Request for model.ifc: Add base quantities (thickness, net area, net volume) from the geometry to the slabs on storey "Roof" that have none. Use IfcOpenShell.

First a look at what the model holds.

```python
import ifcopenshell
import ifcopenshell.util.element
import ifcopenshell.util.unit

model = ifcopenshell.open("model.ifc")
print(model.schema)
for unit_type in ("LENGTHUNIT", "AREAUNIT", "VOLUMEUNIT"):
    print(unit_type, ifcopenshell.util.unit.calculate_unit_scale(model, unit_type))
storey = next(s for s in model.by_type("IfcBuildingStorey") if s.Name == "Roof")
slabs = [e for e in ifcopenshell.util.element.get_decomposition(storey) if e.is_a("IfcSlab")]
for e in sorted(slabs, key=lambda e: e.id()):
    print(e.id(), e.is_a(), e.Name, list(ifcopenshell.util.element.get_psets(e, qtos_only=True)), sep=" | ")
```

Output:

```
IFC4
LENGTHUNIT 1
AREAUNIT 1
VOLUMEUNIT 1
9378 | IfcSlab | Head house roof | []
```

```python
import ifcopenshell
import ifcopenshell.api.pset
import ifcopenshell.geom
import ifcopenshell.util.element
import ifcopenshell.util.shape
import ifcopenshell.util.unit

model = ifcopenshell.open("model.ifc")
unit_scale = ifcopenshell.util.unit.calculate_unit_scale(model)
area_scale = ifcopenshell.util.unit.calculate_unit_scale(model, "AREAUNIT")
volume_scale = ifcopenshell.util.unit.calculate_unit_scale(model, "VOLUMEUNIT")
settings = ifcopenshell.geom.settings()

storey = next(s for s in model.by_type("IfcBuildingStorey") if s.Name == "Roof")
slabs = [e for e in ifcopenshell.util.element.get_decomposition(storey) if e.is_a("IfcSlab")]

for e in sorted(slabs, key=lambda e: e.id()):
    if ifcopenshell.util.element.get_psets(e, qtos_only=True, should_inherit=False):
        continue
    # Geometry comes back in metres, in the element's own axes.
    shape = ifcopenshell.geom.create_shape(settings, e)
    values = {
        "Width": ifcopenshell.util.shape.get_z(shape.geometry) / unit_scale,
        "NetArea": ifcopenshell.util.shape.get_footprint_area(shape.geometry) / area_scale,
        "NetVolume": ifcopenshell.util.shape.get_volume(shape.geometry) / volume_scale,
    }
    qto = ifcopenshell.api.pset.add_qto(model, product=e, name="Qto_SlabBaseQuantities")
    ifcopenshell.api.pset.edit_qto(model, qto=qto, properties=values)
    print(e.id(), {k: round(v, 3) for k, v in values.items()})

model.write("model_updated.ifc")
```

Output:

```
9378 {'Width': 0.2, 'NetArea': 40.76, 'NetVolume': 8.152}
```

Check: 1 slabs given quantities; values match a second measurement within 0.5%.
